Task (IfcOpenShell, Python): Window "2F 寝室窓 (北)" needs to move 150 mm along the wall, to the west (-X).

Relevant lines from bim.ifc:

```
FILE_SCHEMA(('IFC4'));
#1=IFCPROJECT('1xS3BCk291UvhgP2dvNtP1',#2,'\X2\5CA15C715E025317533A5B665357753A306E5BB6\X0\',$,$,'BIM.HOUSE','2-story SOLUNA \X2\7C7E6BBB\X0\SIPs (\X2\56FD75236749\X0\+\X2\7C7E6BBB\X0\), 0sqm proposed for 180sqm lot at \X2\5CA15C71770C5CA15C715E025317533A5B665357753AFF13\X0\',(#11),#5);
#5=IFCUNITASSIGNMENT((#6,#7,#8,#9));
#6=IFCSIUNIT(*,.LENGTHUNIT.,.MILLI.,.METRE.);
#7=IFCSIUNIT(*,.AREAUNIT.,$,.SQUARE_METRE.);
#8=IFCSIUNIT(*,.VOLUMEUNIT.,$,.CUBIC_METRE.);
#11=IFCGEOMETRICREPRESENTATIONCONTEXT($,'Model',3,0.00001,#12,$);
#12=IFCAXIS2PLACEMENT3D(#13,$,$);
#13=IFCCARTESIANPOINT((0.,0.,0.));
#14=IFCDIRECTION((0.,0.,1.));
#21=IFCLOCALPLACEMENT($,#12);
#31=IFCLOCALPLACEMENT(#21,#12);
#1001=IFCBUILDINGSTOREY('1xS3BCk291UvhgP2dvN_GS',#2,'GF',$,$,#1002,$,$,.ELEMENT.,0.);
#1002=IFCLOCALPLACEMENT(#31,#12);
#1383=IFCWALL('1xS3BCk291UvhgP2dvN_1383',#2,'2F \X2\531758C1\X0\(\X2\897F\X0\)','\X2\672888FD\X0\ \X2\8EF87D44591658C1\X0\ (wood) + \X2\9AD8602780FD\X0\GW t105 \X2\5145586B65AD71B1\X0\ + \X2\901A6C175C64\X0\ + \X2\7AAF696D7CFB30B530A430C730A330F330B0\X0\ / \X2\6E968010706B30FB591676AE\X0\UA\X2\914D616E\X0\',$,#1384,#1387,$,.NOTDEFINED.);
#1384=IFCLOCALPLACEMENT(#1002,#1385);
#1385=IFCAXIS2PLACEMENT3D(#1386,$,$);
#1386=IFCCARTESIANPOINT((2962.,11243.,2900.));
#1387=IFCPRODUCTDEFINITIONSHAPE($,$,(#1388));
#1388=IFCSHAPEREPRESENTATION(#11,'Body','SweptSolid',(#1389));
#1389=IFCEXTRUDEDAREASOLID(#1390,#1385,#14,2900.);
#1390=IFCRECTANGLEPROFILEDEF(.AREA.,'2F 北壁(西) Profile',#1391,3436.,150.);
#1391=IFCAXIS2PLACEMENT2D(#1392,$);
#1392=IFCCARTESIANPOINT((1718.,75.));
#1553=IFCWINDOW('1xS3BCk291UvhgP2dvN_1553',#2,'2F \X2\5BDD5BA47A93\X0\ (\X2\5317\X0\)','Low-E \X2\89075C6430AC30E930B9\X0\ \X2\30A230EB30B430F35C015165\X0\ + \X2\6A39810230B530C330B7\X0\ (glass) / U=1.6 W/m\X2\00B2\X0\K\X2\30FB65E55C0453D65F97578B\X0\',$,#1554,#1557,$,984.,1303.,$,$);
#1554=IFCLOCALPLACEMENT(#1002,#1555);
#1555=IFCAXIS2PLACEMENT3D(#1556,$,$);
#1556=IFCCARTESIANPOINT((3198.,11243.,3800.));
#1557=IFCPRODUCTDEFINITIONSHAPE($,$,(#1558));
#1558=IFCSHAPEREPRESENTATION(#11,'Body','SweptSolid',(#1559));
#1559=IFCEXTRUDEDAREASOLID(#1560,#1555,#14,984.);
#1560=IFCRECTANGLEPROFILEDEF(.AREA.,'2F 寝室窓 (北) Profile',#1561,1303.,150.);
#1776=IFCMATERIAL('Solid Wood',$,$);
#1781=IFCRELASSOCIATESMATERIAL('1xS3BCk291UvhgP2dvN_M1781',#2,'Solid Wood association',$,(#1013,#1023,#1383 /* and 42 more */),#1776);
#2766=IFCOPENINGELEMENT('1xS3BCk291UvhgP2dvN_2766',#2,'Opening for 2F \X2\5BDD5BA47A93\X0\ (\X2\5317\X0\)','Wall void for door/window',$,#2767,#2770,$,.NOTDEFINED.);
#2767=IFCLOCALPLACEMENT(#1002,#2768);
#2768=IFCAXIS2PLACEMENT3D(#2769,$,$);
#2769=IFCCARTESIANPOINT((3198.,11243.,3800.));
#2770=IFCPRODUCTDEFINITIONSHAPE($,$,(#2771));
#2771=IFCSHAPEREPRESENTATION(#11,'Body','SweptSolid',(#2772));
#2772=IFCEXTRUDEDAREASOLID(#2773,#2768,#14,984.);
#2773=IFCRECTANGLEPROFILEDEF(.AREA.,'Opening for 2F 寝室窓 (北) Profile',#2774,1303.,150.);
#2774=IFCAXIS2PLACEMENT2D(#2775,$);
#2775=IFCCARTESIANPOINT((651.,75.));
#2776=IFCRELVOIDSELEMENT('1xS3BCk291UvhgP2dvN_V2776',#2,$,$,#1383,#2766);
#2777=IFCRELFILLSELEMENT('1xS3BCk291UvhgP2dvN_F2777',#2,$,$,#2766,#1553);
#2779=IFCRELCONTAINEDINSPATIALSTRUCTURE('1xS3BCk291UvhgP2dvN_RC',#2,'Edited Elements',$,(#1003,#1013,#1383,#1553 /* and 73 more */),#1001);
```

```python
import ifcopenshell
import ifcopenshell.api.geometry
import ifcopenshell.util.placement

model = ifcopenshell.open("bim.ifc")

window = model.by_guid("1xS3BCk291UvhgP2dvN_1553")
opening = window.FillsVoids[0].RelatingOpeningElement
wall = opening.VoidsElements[0].RelatingBuildingElement

wall_matrix = ifcopenshell.util.placement.get_local_placement(wall.ObjectPlacement)
shift = wall_matrix[:3, 0] * -150.0
before = ifcopenshell.util.placement.get_local_placement(window.ObjectPlacement)[:3, 3].copy()

# The window is not placed relative to its opening, so move both.
for product in (opening, window):
    matrix = ifcopenshell.util.placement.get_local_placement(product.ObjectPlacement)
    matrix[:3, 3] += shift
    ifcopenshell.api.geometry.edit_object_placement(model, product=product, matrix=matrix, is_si=False)

after = ifcopenshell.util.placement.get_local_placement(window.ObjectPlacement)[:3, 3]
print("window moved by", (after - before).round(3) + 0.0)

model.write("bim_updated.ifc")
```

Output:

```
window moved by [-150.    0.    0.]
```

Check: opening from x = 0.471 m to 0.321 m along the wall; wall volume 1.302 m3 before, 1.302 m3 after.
